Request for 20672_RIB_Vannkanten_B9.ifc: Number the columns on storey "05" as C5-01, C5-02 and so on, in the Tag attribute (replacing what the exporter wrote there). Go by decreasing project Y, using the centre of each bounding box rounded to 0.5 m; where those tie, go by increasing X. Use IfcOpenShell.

First a look at what the model holds.

```python
import ifcopenshell
import ifcopenshell.util.element
import ifcopenshell.util.placement

model = ifcopenshell.open("20672_RIB_Vannkanten_B9.ifc")
print(model.schema)
storey = next(s for s in model.by_type("IfcBuildingStorey") if s.Name == "05")
columns = [e for e in ifcopenshell.util.element.get_decomposition(storey) if e.is_a("IfcColumn")]
for e in sorted(columns, key=lambda e: e.id()):
    origin = ifcopenshell.util.placement.get_local_placement(e.ObjectPlacement)[:3, 3]
    print(e.id(), e.Tag, e.Name, origin.round(2) + 0.0, sep=" | ")
```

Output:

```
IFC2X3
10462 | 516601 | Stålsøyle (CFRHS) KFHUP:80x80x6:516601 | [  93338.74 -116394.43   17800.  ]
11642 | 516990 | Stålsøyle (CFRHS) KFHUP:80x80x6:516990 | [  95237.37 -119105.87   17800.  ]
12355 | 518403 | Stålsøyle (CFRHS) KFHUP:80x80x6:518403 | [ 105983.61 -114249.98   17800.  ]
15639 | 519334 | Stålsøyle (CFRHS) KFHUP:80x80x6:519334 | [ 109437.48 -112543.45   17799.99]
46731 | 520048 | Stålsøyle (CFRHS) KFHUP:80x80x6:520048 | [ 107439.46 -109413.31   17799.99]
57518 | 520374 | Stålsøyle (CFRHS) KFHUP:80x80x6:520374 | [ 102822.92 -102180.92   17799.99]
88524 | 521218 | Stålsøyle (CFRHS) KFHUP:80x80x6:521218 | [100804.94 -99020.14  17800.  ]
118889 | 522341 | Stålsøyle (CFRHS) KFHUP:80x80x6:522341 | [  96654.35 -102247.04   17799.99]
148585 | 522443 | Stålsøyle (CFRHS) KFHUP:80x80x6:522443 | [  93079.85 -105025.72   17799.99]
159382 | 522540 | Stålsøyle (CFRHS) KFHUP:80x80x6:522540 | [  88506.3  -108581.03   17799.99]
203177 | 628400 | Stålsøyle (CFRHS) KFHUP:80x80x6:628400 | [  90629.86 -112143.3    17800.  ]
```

```python
import ifcopenshell
import ifcopenshell.geom
import ifcopenshell.util.element
import ifcopenshell.util.shape

model = ifcopenshell.open("20672_RIB_Vannkanten_B9.ifc")
settings = ifcopenshell.geom.settings()
settings.set("use-world-coords", True)


def centre(element):
    shape = ifcopenshell.geom.create_shape(settings, element)
    return ifcopenshell.util.shape.get_bbox_centroid(shape.geometry)


storey = next(s for s in model.by_type("IfcBuildingStorey") if s.Name == "05")
columns = [e for e in ifcopenshell.util.element.get_decomposition(storey) if e.is_a("IfcColumn")]

# Insertion points can sit at a corner or the storey origin, so sort by the geometry (in metres).
centres = {e: centre(e) for e in columns}
columns.sort(key=lambda e: (-round(centres[e][1] / 0.5), centres[e][0]))

for i, e in enumerate(columns, start=1):
    number = f"C5-{i:02d}"
    e.Tag = number
    print(e.id(), number)

model.write("20672_RIB_Vannkanten_B9_edited.ifc")
```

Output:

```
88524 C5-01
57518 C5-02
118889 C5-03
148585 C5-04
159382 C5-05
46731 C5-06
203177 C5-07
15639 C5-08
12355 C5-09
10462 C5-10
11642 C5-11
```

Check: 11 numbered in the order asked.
